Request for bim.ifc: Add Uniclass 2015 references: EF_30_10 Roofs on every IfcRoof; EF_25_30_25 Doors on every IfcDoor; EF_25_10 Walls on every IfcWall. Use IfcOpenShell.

First a look at what the model holds.

```python
import ifcopenshell

model = ifcopenshell.open("bim.ifc")
print(model.schema)
print("classifications:", [c.Name for c in model.by_type("IfcClassification")])
for ifc_class in ("IfcDoor", "IfcRoof", "IfcStair", "IfcWall", "IfcWindow"):
    print(ifc_class, len(model.by_type(ifc_class)))
```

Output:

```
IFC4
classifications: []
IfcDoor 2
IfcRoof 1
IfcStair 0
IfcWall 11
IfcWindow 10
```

```python
import ifcopenshell
import ifcopenshell.api.classification

model = ifcopenshell.open("bim.ifc")

system = ifcopenshell.api.classification.add_classification(model, classification="Uniclass 2015")

codes = {
    "IfcRoof": ("EF_30_10", "Roofs"),
    "IfcDoor": ("EF_25_30_25", "Doors"),
    "IfcWall": ("EF_25_10", "Walls"),
}
for ifc_class, (code, name) in codes.items():
    products = model.by_type(ifc_class)
    ifcopenshell.api.classification.add_reference(
        model, products=products, classification=system, identification=code, name=name
    )
    print(code, len(products))

model.write("bim_v2.ifc")
```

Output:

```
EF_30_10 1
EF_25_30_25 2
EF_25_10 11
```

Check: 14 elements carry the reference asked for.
